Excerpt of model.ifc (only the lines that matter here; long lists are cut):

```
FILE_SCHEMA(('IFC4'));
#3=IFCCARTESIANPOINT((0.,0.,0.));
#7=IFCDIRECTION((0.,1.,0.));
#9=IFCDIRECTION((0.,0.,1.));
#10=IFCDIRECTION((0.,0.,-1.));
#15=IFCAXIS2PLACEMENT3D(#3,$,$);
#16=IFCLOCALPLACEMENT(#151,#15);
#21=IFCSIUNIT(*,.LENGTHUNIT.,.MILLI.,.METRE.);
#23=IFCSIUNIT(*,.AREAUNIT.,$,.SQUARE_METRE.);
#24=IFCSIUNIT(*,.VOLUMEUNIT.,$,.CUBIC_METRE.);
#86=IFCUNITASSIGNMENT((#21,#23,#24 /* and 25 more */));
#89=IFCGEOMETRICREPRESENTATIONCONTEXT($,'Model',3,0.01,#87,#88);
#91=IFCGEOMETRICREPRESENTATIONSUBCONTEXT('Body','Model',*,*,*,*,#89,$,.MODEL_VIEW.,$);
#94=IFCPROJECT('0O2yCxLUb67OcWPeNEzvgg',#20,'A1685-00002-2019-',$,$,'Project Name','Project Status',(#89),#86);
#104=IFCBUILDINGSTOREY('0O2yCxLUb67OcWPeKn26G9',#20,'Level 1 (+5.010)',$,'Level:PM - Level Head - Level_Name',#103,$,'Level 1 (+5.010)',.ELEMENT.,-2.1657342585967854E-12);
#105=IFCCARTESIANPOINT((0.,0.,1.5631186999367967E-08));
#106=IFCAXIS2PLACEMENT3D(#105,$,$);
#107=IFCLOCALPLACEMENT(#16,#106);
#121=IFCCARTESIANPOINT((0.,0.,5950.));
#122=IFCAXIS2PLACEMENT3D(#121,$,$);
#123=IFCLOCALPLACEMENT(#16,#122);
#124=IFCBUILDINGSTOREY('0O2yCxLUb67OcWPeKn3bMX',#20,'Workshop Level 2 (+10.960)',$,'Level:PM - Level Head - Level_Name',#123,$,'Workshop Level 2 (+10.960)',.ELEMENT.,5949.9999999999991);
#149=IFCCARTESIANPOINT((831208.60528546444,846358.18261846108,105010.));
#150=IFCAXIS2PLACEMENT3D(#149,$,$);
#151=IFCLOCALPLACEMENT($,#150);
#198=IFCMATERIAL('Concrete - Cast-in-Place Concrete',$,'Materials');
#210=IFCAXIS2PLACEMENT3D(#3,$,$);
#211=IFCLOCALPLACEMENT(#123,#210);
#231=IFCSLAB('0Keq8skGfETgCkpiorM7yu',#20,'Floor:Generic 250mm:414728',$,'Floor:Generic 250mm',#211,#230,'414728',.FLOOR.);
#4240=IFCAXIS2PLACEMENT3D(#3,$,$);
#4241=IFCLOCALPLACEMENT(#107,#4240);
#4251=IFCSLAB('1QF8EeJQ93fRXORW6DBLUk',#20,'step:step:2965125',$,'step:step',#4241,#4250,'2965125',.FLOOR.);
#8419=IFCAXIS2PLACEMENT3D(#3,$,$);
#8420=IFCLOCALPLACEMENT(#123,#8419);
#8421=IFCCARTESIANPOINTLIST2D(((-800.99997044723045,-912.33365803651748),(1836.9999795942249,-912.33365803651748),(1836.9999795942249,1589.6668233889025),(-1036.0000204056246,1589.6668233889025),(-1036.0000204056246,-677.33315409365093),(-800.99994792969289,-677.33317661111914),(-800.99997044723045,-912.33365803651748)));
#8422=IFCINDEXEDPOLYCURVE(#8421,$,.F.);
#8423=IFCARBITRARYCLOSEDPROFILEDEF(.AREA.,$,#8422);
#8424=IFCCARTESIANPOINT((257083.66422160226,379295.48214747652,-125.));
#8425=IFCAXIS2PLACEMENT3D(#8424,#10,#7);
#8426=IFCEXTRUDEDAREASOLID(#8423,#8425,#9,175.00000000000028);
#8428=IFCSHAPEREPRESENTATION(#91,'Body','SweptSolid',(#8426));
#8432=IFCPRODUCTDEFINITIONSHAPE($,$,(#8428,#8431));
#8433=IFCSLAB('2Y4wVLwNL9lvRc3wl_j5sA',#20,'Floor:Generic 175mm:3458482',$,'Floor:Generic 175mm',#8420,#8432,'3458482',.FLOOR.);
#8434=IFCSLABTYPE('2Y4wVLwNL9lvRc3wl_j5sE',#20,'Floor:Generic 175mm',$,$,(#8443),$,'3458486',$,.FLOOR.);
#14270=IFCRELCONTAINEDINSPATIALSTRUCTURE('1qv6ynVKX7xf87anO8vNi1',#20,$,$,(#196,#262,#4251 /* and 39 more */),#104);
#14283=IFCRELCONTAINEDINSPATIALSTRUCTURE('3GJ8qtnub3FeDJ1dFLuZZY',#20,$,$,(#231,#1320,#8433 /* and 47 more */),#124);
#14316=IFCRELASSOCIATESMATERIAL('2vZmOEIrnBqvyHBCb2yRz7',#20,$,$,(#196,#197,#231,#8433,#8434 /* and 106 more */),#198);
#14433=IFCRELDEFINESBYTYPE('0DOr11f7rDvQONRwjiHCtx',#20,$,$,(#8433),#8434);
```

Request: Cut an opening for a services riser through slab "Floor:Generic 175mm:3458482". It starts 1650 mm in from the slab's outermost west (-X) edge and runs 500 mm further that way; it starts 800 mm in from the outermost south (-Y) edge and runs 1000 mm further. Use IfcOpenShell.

```python
import numpy as np
import ifcopenshell
import ifcopenshell.api.feature
import ifcopenshell.api.geometry
import ifcopenshell.api.root
import ifcopenshell.geom
import ifcopenshell.util.placement
import ifcopenshell.util.representation
import ifcopenshell.util.shape
import ifcopenshell.util.unit

model = ifcopenshell.open("model.ifc")
unit_scale = ifcopenshell.util.unit.calculate_unit_scale(model)
settings = ifcopenshell.geom.settings()


def volume(element):
    """Net volume in cubic metres, openings subtracted."""
    shape = ifcopenshell.geom.create_shape(settings, element)
    return ifcopenshell.util.shape.get_volume(shape.geometry)


slab = model.by_id(8433)
before = volume(slab)

# Extent in the slab's own axes, in metres. The edges named are its -X and -Y sides.
slab_shape = ifcopenshell.geom.create_shape(settings, slab)
vertices = ifcopenshell.util.shape.get_vertices(slab_shape.geometry)
x_min, y_min, bottom = vertices.min(axis=0)
top = vertices[:, 2].max()

opening = ifcopenshell.api.root.create_entity(model, ifc_class="IfcOpeningElement", name="Services riser opening", predefined_type="OPENING")
context = ifcopenshell.util.representation.get_context(model, "Model", "Body", "MODEL_VIEW")
width, depth = 0.5, 1
outline = [(0.0, 0.0), (width, 0.0), (width, depth), (0.0, depth), (0.0, 0.0)]
# Overshoot both faces by 50 mm so the cut is clean.
shape = ifcopenshell.api.geometry.add_slab_representation(
    model, context=context, depth=top - bottom + 0.1, polyline=outline
)
ifcopenshell.api.geometry.assign_representation(model, product=opening, representation=shape)

matrix = ifcopenshell.util.placement.get_local_placement(slab.ObjectPlacement)
matrix[:, 3] = matrix @ np.append(np.array([x_min + 1.65, y_min + 0.8, bottom - 0.05]) / unit_scale, 1.0)
ifcopenshell.api.geometry.edit_object_placement(model, product=opening, matrix=matrix, is_si=False)
ifcopenshell.api.feature.add_feature(model, feature=opening, element=slab)

after = volume(slab)

print(f"slab volume {before:.3f} -> {after:.3f} m3")

model.write("model_rev.ifc")
```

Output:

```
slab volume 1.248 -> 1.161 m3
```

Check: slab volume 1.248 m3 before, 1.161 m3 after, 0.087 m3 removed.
